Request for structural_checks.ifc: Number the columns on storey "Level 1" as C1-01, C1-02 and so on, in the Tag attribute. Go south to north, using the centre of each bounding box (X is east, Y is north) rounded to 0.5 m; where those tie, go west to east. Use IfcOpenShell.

First a look at what the model holds.

```python
import ifcopenshell
import ifcopenshell.util.element
import ifcopenshell.util.placement

model = ifcopenshell.open("structural_checks.ifc")
print(model.schema)
storey = next(s for s in model.by_type("IfcBuildingStorey") if s.Name == "Level 1")
columns = [e for e in ifcopenshell.util.element.get_decomposition(storey) if e.is_a("IfcColumn")]
for e in sorted(columns, key=lambda e: e.id()):
    origin = ifcopenshell.util.placement.get_local_placement(e.ObjectPlacement)[:3, 3]
    print(e.id(), e.Tag, e.Name, origin.round(2) + 0.0, sep=" | ")
```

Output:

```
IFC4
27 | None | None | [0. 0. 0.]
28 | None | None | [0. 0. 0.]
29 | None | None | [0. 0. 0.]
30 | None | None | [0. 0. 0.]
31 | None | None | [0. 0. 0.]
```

```python
import ifcopenshell
import ifcopenshell.geom
import ifcopenshell.util.element
import ifcopenshell.util.shape

model = ifcopenshell.open("structural_checks.ifc")
settings = ifcopenshell.geom.settings()
settings.set("use-world-coords", True)


def centre(element):
    shape = ifcopenshell.geom.create_shape(settings, element)
    return ifcopenshell.util.shape.get_bbox_centroid(shape.geometry)


storey = next(s for s in model.by_type("IfcBuildingStorey") if s.Name == "Level 1")
columns = [e for e in ifcopenshell.util.element.get_decomposition(storey) if e.is_a("IfcColumn")]

# Insertion points can sit at a corner or the storey origin, so sort by the geometry (in metres).
centres = {e: centre(e) for e in columns}
columns.sort(key=lambda e: (round(centres[e][1] / 0.5), centres[e][0]))

for i, e in enumerate(columns, start=1):
    number = f"C1-{i:02d}"
    e.Tag = number
    print(e.id(), number)

model.write("structural_checks_v2.ifc")
```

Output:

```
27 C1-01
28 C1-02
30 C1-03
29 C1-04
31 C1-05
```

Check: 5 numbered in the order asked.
